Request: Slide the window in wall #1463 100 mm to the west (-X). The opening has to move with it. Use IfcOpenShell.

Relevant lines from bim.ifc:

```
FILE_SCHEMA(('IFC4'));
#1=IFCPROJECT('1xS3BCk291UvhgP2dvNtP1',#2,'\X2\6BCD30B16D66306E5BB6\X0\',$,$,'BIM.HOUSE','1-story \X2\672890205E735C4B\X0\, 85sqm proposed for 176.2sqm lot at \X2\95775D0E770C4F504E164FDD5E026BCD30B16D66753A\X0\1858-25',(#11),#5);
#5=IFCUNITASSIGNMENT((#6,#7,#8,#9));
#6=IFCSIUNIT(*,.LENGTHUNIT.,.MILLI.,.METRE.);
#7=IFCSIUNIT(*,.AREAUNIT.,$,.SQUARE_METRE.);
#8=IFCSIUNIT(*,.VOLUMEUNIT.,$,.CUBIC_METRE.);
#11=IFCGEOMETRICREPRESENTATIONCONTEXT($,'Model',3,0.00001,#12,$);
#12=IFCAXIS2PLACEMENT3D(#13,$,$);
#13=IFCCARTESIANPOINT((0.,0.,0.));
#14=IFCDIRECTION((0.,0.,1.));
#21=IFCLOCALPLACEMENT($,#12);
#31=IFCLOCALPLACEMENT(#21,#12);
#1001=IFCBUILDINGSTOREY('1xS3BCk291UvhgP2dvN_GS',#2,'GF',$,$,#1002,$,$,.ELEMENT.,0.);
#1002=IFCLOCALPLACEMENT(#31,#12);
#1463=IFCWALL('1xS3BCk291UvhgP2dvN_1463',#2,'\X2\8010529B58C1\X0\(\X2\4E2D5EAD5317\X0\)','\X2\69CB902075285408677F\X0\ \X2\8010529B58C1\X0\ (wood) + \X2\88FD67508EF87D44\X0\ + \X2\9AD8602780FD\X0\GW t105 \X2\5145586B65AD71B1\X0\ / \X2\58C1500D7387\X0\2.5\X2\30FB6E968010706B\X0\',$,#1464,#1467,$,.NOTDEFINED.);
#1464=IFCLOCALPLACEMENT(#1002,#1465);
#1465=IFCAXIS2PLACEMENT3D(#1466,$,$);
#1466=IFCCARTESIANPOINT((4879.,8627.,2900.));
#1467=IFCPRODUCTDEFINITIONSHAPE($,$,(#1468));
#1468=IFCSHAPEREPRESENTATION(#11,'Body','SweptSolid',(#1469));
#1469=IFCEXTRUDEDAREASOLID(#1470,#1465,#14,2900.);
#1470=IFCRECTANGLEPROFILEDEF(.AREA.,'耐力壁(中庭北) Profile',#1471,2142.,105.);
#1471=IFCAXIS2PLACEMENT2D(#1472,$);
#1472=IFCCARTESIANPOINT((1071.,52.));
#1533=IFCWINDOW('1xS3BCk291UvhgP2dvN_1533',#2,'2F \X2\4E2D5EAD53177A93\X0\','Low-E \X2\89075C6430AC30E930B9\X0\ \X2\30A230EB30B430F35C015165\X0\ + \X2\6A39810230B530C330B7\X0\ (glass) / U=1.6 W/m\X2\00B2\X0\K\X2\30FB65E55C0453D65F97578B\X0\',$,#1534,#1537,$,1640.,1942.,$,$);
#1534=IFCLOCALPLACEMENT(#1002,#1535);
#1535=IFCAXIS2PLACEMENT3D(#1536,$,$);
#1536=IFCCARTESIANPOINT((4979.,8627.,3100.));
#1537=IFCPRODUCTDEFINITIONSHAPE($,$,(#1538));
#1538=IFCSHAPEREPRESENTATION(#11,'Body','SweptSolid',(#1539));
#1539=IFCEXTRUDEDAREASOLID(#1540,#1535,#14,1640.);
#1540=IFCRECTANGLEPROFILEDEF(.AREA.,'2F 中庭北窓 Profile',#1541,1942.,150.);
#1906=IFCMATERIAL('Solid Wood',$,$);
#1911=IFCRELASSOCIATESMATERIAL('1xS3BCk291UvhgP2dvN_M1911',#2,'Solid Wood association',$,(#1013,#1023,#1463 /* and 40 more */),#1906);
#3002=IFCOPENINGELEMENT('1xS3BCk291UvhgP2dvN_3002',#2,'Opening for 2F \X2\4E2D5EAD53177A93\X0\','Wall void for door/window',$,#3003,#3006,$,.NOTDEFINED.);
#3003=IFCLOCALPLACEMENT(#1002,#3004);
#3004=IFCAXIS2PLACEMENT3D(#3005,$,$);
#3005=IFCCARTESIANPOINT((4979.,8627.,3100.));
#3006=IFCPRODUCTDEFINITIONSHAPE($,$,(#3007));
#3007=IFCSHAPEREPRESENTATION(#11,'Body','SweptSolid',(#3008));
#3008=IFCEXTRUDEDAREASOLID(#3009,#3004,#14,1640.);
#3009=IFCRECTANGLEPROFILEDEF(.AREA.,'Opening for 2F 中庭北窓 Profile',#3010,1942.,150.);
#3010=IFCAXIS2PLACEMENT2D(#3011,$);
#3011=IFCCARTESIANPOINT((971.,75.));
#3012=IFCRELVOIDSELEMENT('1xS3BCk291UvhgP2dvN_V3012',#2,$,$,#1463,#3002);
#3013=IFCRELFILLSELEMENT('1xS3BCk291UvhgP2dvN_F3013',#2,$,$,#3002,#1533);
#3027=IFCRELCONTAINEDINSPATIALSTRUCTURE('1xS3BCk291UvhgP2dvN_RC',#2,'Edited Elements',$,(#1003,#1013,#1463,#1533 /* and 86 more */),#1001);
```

```python
import ifcopenshell
import ifcopenshell.api.geometry
import ifcopenshell.util.placement
import ifcopenshell.util.unit

model = ifcopenshell.open("bim.ifc")
unit_scale = ifcopenshell.util.unit.calculate_unit_scale(model)

window = model.by_guid("1xS3BCk291UvhgP2dvN_1533")
opening = window.FillsVoids[0].RelatingOpeningElement
wall = opening.VoidsElements[0].RelatingBuildingElement

wall_matrix = ifcopenshell.util.placement.get_local_placement(wall.ObjectPlacement)
shift = wall_matrix[:3, 0] * -0.1 / unit_scale
before = ifcopenshell.util.placement.get_local_placement(window.ObjectPlacement)[:3, 3].copy()

# The window is not placed relative to its opening, so move both.
for product in (opening, window):
    matrix = ifcopenshell.util.placement.get_local_placement(product.ObjectPlacement)
    matrix[:3, 3] += shift
    ifcopenshell.api.geometry.edit_object_placement(model, product=product, matrix=matrix, is_si=False)

after = ifcopenshell.util.placement.get_local_placement(window.ObjectPlacement)[:3, 3]
print("window moved by", (after - before).round(3) + 0.0)

model.write("bim_v2.ifc")
```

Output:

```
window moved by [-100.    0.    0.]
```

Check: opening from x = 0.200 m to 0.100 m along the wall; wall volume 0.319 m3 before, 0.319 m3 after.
